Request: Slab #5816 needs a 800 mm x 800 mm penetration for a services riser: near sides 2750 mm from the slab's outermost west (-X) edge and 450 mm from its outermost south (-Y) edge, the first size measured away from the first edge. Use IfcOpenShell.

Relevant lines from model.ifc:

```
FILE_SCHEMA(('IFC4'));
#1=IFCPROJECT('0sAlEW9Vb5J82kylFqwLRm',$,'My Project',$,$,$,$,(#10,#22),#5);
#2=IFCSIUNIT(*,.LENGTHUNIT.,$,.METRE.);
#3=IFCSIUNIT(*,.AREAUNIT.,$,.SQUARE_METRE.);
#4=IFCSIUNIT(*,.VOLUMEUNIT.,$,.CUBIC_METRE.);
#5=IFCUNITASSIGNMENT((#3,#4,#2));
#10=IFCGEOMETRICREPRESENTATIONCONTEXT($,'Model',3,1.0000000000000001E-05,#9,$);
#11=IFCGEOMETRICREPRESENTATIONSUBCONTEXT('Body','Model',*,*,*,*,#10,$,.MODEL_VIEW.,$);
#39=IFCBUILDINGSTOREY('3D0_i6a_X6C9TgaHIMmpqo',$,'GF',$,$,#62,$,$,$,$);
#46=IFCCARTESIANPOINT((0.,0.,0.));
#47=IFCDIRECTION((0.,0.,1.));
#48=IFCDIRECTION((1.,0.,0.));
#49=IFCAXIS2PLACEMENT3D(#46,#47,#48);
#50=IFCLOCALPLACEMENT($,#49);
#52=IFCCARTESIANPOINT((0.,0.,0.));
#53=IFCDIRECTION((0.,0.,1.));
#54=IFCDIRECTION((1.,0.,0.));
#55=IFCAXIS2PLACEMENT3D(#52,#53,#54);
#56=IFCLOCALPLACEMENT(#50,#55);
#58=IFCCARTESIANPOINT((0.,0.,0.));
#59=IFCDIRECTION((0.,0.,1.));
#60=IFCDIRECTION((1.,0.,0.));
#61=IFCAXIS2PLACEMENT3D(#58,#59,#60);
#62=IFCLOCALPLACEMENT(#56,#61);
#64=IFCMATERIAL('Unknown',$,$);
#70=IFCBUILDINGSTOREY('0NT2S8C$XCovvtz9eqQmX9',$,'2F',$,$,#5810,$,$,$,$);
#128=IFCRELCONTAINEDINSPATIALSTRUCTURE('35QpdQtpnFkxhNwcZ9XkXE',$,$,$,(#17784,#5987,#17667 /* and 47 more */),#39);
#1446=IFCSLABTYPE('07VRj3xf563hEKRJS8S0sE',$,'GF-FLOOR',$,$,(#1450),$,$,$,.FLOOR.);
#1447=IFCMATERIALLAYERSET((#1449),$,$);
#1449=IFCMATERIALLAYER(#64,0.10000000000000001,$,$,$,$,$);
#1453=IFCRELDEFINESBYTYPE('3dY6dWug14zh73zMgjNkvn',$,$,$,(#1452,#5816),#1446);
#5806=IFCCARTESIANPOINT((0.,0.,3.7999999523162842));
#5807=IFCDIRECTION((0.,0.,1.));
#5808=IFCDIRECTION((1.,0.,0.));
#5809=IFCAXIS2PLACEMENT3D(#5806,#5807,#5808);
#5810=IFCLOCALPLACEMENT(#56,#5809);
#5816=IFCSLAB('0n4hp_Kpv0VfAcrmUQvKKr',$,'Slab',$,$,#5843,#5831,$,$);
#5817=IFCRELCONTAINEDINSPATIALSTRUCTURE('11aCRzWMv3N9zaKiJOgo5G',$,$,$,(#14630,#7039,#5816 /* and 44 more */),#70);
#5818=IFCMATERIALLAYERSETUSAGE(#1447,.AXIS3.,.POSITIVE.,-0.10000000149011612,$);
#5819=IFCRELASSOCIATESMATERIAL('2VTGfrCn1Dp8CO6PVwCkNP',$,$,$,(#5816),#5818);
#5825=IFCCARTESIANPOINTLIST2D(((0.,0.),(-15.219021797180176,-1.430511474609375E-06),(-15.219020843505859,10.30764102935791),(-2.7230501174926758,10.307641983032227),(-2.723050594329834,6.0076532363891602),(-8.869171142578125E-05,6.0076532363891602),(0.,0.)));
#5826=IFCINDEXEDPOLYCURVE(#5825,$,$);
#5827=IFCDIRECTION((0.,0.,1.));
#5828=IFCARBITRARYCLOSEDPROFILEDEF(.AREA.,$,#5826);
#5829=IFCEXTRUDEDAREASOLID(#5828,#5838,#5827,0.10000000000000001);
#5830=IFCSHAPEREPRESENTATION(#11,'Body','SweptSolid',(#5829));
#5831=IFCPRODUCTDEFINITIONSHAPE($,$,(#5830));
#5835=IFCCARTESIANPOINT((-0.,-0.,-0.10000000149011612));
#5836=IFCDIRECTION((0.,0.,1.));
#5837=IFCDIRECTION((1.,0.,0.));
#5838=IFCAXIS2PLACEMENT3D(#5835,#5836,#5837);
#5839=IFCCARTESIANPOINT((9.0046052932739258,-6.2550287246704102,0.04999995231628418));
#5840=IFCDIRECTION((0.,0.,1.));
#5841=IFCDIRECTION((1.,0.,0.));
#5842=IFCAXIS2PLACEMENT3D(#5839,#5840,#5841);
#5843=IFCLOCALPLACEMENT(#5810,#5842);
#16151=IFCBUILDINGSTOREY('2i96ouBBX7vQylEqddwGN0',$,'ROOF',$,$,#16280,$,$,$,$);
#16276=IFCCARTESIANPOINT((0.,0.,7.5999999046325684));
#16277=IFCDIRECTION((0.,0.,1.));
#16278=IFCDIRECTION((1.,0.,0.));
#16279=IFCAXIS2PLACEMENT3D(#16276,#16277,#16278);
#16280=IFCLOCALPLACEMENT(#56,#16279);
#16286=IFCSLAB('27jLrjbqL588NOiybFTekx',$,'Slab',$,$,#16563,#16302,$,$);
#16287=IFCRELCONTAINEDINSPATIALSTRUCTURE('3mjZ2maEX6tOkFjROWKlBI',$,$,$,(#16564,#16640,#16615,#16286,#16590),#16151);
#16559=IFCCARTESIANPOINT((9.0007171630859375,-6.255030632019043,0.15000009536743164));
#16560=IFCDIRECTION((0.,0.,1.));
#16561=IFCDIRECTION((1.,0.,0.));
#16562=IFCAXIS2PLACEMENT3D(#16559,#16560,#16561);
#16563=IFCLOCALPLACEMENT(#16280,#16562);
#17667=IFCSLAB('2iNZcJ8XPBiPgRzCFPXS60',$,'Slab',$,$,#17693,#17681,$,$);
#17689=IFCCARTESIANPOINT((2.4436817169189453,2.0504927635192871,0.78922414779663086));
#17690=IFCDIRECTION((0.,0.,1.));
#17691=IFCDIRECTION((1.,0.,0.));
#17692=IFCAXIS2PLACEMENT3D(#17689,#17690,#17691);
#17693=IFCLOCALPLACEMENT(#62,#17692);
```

```python
import numpy as np
import ifcopenshell
import ifcopenshell.api.feature
import ifcopenshell.api.geometry
import ifcopenshell.api.root
import ifcopenshell.geom
import ifcopenshell.util.placement
import ifcopenshell.util.representation
import ifcopenshell.util.shape
import ifcopenshell.util.unit

model = ifcopenshell.open("model.ifc")
unit_scale = ifcopenshell.util.unit.calculate_unit_scale(model)
settings = ifcopenshell.geom.settings()


def volume(element):
    """Net volume in cubic metres, openings subtracted."""
    shape = ifcopenshell.geom.create_shape(settings, element)
    return ifcopenshell.util.shape.get_volume(shape.geometry)


slab = model.by_id(5816)
before = volume(slab)

# Extent in the slab's own axes, in metres. The edges named are its -X and -Y sides.
slab_shape = ifcopenshell.geom.create_shape(settings, slab)
vertices = ifcopenshell.util.shape.get_vertices(slab_shape.geometry)
x_min, y_min, bottom = vertices.min(axis=0)
top = vertices[:, 2].max()

opening = ifcopenshell.api.root.create_entity(model, ifc_class="IfcOpeningElement", name="Services riser opening", predefined_type="OPENING")
context = ifcopenshell.util.representation.get_context(model, "Model", "Body", "MODEL_VIEW")
width, depth = 0.8, 0.8
outline = [(0.0, 0.0), (width, 0.0), (width, depth), (0.0, depth), (0.0, 0.0)]
# Overshoot both faces by 50 mm so the cut is clean.
shape = ifcopenshell.api.geometry.add_slab_representation(
    model, context=context, depth=top - bottom + 0.1, polyline=outline
)
ifcopenshell.api.geometry.assign_representation(model, product=opening, representation=shape)

matrix = ifcopenshell.util.placement.get_local_placement(slab.ObjectPlacement)
matrix[:, 3] = matrix @ np.append(np.array([x_min + 2.75, y_min + 0.45, bottom - 0.05]) / unit_scale, 1.0)
ifcopenshell.api.geometry.edit_object_placement(model, product=opening, matrix=matrix, is_si=False)
ifcopenshell.api.feature.add_feature(model, feature=opening, element=slab)

after = volume(slab)

print(f"slab volume {before:.3f} -> {after:.3f} m3")

model.write("model_rev.ifc")
```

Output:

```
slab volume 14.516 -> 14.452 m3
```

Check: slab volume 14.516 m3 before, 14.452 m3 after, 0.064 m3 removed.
